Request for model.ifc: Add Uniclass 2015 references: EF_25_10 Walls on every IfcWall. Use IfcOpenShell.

First a look at what the model holds.

```python
import ifcopenshell

model = ifcopenshell.open("model.ifc")
print(model.schema)
print("classifications:", [c.Name for c in model.by_type("IfcClassification")])
for ifc_class in ("IfcDoor", "IfcRoof", "IfcStair", "IfcWall", "IfcWindow"):
    print(ifc_class, len(model.by_type(ifc_class)))
```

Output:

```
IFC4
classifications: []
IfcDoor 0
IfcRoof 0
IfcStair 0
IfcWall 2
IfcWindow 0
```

```python
import ifcopenshell
import ifcopenshell.api.classification

model = ifcopenshell.open("model.ifc")

system = ifcopenshell.api.classification.add_classification(model, classification="Uniclass 2015")

codes = {
    "IfcWall": ("EF_25_10", "Walls"),
}
for ifc_class, (code, name) in codes.items():
    products = model.by_type(ifc_class)
    ifcopenshell.api.classification.add_reference(
        model, products=products, classification=system, identification=code, name=name
    )
    print(code, len(products))

model.write("model_edited.ifc")
```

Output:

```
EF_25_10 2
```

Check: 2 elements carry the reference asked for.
